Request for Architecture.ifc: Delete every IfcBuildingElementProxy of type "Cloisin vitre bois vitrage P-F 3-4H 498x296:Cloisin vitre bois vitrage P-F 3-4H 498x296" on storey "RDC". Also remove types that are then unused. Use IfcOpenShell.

First a look at what the model holds.

```python
import ifcopenshell
import ifcopenshell.util.element

model = ifcopenshell.open("Architecture.ifc")
print(model.schema)
storey = next(s for s in model.by_type("IfcBuildingStorey") if s.Name == "RDC")
proxies = [e for e in ifcopenshell.util.element.get_decomposition(storey) if e.is_a("IfcBuildingElementProxy")]
seen = {}
for e in proxies:
    element_type = ifcopenshell.util.element.get_type(e)
    name = element_type.Name if element_type not in (None, e) else None
    seen[name] = seen.get(name, 0) + 1
for name, count in sorted(seen.items(), key=str):
    print(count, "x", name)
```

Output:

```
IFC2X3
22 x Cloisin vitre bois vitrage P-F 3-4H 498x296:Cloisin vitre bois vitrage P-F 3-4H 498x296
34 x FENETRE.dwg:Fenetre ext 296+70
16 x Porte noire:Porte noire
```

```python
import ifcopenshell
import ifcopenshell.api.root
import ifcopenshell.util.element

model = ifcopenshell.open("Architecture.ifc")

storey = next(s for s in model.by_type("IfcBuildingStorey") if s.Name == "RDC")
proxies = [e for e in ifcopenshell.util.element.get_decomposition(storey) if e.is_a("IfcBuildingElementProxy")]
targets = [e for e in proxies if (t := ifcopenshell.util.element.get_type(e)) not in (None, e) and t.Name == "Cloisin vitre bois vitrage P-F 3-4H 498x296:Cloisin vitre bois vitrage P-F 3-4H 498x296"]
types = {ifcopenshell.util.element.get_type(e) for e in targets} - {None, *targets}

for e in targets:
    ifcopenshell.api.root.remove_product(model, product=e)
print(len(targets), "removed")

unused = [t for t in types if not ifcopenshell.util.element.get_types(t)]
for t in unused:
    ifcopenshell.api.root.remove_product(model, product=t)
print(len(unused), "unused types removed")

model.write("Architecture_edited.ifc")
```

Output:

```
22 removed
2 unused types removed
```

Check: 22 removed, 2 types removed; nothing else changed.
